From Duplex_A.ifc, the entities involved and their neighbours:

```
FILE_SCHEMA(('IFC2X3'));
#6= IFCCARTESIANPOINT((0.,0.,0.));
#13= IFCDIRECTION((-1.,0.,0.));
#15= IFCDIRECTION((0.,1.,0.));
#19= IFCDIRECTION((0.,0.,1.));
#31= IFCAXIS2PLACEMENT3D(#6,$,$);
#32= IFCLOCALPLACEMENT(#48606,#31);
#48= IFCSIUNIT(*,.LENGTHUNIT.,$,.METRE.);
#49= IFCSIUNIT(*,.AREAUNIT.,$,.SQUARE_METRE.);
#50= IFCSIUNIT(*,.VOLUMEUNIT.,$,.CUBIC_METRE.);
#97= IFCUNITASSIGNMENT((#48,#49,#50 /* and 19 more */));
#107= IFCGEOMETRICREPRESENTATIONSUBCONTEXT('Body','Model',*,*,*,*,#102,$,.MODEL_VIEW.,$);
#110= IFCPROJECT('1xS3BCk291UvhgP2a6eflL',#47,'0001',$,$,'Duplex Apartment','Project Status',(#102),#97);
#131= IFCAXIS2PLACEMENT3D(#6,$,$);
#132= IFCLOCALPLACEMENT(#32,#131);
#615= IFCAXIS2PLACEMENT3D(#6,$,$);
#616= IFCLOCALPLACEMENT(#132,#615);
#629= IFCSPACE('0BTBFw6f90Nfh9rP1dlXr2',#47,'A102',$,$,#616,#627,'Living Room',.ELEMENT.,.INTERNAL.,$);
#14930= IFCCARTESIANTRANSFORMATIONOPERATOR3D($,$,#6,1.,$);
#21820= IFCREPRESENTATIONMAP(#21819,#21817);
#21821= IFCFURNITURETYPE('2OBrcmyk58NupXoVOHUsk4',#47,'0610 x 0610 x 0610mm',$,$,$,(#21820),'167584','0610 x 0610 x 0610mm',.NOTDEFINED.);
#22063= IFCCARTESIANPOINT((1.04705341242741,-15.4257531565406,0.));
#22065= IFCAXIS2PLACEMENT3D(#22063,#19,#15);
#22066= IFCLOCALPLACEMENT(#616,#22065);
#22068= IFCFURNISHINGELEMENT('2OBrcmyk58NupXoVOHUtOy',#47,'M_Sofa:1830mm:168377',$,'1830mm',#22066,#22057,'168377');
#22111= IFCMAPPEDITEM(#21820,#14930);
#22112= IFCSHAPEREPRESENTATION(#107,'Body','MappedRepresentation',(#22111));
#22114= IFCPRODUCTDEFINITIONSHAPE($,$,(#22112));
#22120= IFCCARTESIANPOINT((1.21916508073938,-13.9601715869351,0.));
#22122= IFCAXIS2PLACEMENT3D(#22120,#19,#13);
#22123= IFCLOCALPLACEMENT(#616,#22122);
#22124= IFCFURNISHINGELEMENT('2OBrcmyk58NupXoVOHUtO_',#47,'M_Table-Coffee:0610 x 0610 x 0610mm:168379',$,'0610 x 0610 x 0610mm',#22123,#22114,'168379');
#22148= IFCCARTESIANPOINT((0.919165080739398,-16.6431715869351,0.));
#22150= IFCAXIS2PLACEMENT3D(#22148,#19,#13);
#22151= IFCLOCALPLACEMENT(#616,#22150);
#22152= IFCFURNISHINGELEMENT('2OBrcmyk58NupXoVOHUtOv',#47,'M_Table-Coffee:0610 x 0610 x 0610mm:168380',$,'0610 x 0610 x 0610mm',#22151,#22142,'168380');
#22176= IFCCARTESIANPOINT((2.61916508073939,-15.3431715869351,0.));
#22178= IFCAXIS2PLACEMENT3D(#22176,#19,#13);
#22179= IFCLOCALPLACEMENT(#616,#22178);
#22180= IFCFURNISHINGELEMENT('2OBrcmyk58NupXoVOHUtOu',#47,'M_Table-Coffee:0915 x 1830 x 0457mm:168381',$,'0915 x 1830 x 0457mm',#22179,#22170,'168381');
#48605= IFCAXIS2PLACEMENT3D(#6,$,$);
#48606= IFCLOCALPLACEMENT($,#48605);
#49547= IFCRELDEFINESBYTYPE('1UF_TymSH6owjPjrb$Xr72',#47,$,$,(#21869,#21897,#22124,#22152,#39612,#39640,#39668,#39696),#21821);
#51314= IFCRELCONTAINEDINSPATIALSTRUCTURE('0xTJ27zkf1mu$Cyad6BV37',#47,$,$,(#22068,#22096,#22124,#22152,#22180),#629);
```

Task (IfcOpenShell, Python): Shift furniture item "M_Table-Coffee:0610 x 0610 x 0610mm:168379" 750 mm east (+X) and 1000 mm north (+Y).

```python
import ifcopenshell
import ifcopenshell.api.geometry
import ifcopenshell.util.placement
import ifcopenshell.util.unit

model = ifcopenshell.open("Duplex_A.ifc")
unit_scale = ifcopenshell.util.unit.calculate_unit_scale(model)

item = model.by_guid("2OBrcmyk58NupXoVOHUtO_")
matrix = ifcopenshell.util.placement.get_local_placement(item.ObjectPlacement)
matrix[0, 3] += 0.75 / unit_scale
matrix[1, 3] += 1 / unit_scale
ifcopenshell.api.geometry.edit_object_placement(model, product=item, matrix=matrix, is_si=False)

print(ifcopenshell.util.placement.get_local_placement(item.ObjectPlacement).round(3) + 0.0)

model.write("Duplex_A_v2.ifc")
```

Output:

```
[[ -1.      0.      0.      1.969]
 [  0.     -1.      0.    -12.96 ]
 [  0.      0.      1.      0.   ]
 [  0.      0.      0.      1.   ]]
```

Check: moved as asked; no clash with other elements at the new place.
